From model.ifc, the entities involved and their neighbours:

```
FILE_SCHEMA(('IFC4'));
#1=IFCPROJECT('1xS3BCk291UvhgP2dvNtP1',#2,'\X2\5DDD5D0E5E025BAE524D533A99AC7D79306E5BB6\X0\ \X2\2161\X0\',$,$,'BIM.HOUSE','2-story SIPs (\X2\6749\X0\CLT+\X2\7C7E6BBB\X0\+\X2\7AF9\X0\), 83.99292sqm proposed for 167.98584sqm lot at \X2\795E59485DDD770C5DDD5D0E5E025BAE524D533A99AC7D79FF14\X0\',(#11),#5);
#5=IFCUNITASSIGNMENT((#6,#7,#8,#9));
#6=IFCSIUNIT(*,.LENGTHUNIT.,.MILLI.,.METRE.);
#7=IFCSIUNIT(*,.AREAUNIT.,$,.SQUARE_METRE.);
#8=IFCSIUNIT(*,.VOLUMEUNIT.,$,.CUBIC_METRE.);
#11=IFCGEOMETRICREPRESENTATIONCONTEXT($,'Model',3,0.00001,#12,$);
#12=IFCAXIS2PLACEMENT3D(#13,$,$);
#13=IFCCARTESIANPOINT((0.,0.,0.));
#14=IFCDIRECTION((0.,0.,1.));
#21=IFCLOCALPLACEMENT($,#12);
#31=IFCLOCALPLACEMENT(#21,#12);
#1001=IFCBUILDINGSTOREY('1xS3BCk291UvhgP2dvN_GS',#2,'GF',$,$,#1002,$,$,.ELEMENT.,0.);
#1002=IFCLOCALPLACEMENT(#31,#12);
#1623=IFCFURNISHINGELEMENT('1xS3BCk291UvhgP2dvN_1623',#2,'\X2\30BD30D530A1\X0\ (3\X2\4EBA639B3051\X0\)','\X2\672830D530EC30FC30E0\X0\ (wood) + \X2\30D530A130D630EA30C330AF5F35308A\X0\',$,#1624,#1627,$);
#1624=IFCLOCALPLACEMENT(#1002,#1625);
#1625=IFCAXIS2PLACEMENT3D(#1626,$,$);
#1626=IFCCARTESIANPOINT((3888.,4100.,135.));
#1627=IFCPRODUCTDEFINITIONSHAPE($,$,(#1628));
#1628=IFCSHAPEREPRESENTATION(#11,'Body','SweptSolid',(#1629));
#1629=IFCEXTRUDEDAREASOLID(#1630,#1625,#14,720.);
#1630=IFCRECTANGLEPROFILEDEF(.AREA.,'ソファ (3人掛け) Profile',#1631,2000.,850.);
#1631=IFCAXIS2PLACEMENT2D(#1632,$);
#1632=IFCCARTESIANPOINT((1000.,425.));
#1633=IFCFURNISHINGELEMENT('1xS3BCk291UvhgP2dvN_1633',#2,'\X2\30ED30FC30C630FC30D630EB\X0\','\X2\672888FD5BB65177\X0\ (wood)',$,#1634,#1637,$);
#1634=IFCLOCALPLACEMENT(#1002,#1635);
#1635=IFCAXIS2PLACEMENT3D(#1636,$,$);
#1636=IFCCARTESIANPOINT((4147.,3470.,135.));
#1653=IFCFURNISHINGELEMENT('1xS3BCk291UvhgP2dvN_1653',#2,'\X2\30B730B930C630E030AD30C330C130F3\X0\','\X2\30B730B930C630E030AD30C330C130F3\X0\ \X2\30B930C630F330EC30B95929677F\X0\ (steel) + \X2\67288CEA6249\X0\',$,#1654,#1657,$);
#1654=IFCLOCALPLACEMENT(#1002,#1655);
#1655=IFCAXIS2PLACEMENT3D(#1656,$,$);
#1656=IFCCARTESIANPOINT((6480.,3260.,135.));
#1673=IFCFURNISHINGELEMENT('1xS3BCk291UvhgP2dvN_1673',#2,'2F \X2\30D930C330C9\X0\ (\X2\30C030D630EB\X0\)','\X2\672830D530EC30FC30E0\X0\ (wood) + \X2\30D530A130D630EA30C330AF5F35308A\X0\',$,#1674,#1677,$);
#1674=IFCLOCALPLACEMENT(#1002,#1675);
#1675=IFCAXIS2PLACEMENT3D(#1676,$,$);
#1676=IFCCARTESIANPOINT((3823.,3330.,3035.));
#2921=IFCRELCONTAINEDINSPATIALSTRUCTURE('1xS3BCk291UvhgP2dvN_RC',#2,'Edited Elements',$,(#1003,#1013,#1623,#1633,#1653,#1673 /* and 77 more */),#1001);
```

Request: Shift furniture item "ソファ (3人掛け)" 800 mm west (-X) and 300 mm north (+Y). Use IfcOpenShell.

```python
import ifcopenshell
import ifcopenshell.api.geometry
import ifcopenshell.util.placement

model = ifcopenshell.open("model.ifc")

item = model.by_id(1623)
matrix = ifcopenshell.util.placement.get_local_placement(item.ObjectPlacement)
matrix[0, 3] -= 800.0
matrix[1, 3] += 300.0
ifcopenshell.api.geometry.edit_object_placement(model, product=item, matrix=matrix, is_si=False)

print(ifcopenshell.util.placement.get_local_placement(item.ObjectPlacement).round(3) + 0.0)

model.write("model_rev.ifc")
```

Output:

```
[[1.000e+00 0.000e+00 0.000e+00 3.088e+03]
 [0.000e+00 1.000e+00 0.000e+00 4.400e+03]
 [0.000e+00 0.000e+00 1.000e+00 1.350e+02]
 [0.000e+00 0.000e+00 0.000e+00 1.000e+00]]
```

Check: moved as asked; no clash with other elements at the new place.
